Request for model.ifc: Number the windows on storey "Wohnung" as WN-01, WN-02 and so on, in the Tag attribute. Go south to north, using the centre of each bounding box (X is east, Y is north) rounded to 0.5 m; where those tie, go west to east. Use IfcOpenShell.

First a look at what the model holds.

```python
import ifcopenshell
import ifcopenshell.util.element
import ifcopenshell.util.placement

model = ifcopenshell.open("model.ifc")
print(model.schema)
storey = next(s for s in model.by_type("IfcBuildingStorey") if s.Name == "Wohnung")
windows = [e for e in ifcopenshell.util.element.get_decomposition(storey) if e.is_a("IfcWindow")]
for e in sorted(windows, key=lambda e: e.id()):
    origin = ifcopenshell.util.placement.get_local_placement(e.ObjectPlacement)[:3, 3]
    print(e.id(), e.Tag, e.Name, origin.round(2) + 0.0, sep=" | ")
```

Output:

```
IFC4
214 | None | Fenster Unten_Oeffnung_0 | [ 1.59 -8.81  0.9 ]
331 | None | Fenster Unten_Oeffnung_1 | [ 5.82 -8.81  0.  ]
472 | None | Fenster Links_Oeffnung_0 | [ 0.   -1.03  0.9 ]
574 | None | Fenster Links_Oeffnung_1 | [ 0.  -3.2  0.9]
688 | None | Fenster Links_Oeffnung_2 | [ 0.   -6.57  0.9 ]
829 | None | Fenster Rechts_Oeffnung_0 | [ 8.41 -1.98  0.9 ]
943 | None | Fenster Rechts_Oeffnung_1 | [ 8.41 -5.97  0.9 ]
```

```python
import ifcopenshell
import ifcopenshell.geom
import ifcopenshell.util.element
import ifcopenshell.util.shape

model = ifcopenshell.open("model.ifc")
settings = ifcopenshell.geom.settings()
settings.set("use-world-coords", True)


def centre(element):
    shape = ifcopenshell.geom.create_shape(settings, element)
    return ifcopenshell.util.shape.get_bbox_centroid(shape.geometry)


storey = next(s for s in model.by_type("IfcBuildingStorey") if s.Name == "Wohnung")
windows = [e for e in ifcopenshell.util.element.get_decomposition(storey) if e.is_a("IfcWindow")]

# Insertion points can sit at a corner or the storey origin, so sort by the geometry (in metres).
centres = {e: centre(e) for e in windows}
windows.sort(key=lambda e: (round(centres[e][1] / 0.5), centres[e][0]))

for i, e in enumerate(windows, start=1):
    number = f"WN-{i:02d}"
    e.Tag = number
    print(e.id(), number)

model.write("model_v2.ifc")
```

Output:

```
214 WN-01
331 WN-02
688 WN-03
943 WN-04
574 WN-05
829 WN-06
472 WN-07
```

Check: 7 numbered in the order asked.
